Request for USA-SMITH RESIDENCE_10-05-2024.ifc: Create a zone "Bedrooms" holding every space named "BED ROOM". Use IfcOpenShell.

First a look at what the model holds.

```python
import ifcopenshell

model = ifcopenshell.open("USA-SMITH RESIDENCE_10-05-2024.ifc")
print(model.schema)
seen = {}
for space in model.by_type("IfcSpace"):
    seen[space.LongName] = seen.get(space.LongName, 0) + 1
for name, count in sorted(seen.items(), key=str):
    print(count, "x", name)
print("zones:", [z.Name for z in model.by_type("IfcZone")][:20])
```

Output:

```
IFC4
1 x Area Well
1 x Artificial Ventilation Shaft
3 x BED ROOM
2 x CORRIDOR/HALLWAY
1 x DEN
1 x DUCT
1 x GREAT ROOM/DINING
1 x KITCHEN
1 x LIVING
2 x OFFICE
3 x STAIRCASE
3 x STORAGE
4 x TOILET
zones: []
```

```python
import ifcopenshell
import ifcopenshell.api.group
import ifcopenshell.api.root

model = ifcopenshell.open("USA-SMITH RESIDENCE_10-05-2024.ifc")

names = {"BED ROOM"}
spaces = [s for s in model.by_type("IfcSpace") if s.LongName in names]

zone = ifcopenshell.api.root.create_entity(model, ifc_class="IfcZone", name="Bedrooms")
ifcopenshell.api.group.assign_group(model, products=spaces, group=zone)
print(len(spaces), "spaces in", zone.Name)

model.write("USA-SMITH RESIDENCE_10-05-2024-out.ifc")
```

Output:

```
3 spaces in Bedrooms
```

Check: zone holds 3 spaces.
